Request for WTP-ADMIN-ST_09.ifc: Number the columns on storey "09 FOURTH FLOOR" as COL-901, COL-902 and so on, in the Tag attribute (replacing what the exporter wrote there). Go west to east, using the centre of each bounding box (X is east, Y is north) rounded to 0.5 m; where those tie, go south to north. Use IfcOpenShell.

First a look at what the model holds.

```python
import ifcopenshell
import ifcopenshell.util.element
import ifcopenshell.util.placement

model = ifcopenshell.open("WTP-ADMIN-ST_09.ifc")
print(model.schema)
storey = next(s for s in model.by_type("IfcBuildingStorey") if s.Name == "09 FOURTH FLOOR")
columns = [e for e in ifcopenshell.util.element.get_decomposition(storey) if e.is_a("IfcColumn")]
for e in sorted(columns, key=lambda e: e.id()):
    origin = ifcopenshell.util.placement.get_local_placement(e.ObjectPlacement)[:3, 3]
    print(e.id(), e.Tag, e.Name, origin.round(2) + 0.0, sep=" | ")
```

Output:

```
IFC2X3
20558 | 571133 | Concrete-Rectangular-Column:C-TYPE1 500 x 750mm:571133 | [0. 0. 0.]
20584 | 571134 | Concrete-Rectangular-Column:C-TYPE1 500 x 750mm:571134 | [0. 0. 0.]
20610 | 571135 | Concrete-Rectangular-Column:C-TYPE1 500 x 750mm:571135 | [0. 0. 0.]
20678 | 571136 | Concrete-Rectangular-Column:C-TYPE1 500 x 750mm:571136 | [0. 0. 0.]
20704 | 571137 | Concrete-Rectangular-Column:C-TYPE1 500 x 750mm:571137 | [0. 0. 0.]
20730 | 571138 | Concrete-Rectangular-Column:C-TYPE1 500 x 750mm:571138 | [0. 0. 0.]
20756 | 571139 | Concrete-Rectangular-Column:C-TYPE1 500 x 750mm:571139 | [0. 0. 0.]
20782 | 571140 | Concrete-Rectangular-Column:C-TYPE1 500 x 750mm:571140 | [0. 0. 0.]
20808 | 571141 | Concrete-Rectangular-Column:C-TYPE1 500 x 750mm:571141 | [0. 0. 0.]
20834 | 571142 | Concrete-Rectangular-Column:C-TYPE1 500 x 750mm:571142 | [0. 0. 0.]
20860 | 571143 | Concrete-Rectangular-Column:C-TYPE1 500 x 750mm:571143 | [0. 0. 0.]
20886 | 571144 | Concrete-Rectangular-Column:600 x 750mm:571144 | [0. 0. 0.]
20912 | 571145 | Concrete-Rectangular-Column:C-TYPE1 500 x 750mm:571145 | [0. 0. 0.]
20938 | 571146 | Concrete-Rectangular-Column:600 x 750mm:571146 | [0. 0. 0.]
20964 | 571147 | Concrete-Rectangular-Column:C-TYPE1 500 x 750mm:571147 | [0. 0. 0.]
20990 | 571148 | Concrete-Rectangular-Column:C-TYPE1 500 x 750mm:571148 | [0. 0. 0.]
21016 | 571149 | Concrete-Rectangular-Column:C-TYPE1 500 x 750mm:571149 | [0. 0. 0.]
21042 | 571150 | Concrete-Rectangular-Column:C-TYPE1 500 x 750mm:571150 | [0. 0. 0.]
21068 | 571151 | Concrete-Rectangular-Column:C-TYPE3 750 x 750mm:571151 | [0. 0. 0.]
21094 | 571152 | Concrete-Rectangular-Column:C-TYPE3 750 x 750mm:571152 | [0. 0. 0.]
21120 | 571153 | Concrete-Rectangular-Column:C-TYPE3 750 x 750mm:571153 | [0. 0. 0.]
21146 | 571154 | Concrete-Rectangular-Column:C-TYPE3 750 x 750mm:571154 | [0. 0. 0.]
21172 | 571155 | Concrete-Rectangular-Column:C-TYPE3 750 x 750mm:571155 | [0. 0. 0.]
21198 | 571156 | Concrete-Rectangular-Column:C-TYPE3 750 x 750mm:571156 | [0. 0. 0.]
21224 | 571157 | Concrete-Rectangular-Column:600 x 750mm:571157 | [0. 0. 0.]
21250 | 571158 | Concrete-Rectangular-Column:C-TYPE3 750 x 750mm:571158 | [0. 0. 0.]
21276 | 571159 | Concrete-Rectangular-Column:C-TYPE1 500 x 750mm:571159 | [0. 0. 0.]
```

```python
import ifcopenshell
import ifcopenshell.geom
import ifcopenshell.util.element
import ifcopenshell.util.shape

model = ifcopenshell.open("WTP-ADMIN-ST_09.ifc")
settings = ifcopenshell.geom.settings()
settings.set("use-world-coords", True)


def centre(element):
    shape = ifcopenshell.geom.create_shape(settings, element)
    return ifcopenshell.util.shape.get_bbox_centroid(shape.geometry)


storey = next(s for s in model.by_type("IfcBuildingStorey") if s.Name == "09 FOURTH FLOOR")
columns = [e for e in ifcopenshell.util.element.get_decomposition(storey) if e.is_a("IfcColumn")]

# Insertion points can sit at a corner or the storey origin, so sort by the geometry (in metres).
centres = {e: centre(e) for e in columns}
columns.sort(key=lambda e: (round(centres[e][0] / 0.5), centres[e][1]))

for i, e in enumerate(columns, start=1):
    number = f"COL-9{i:02d}"
    e.Tag = number
    print(e.id(), number)

model.write("WTP-ADMIN-ST_09_edited.ifc")
```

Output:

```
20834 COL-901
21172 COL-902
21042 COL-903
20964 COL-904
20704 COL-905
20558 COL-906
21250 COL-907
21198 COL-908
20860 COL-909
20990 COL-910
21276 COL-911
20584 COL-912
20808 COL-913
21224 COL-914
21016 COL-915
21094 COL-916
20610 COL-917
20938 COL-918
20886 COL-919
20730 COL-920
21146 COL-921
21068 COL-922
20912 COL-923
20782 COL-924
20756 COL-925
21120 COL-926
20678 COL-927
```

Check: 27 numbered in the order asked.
